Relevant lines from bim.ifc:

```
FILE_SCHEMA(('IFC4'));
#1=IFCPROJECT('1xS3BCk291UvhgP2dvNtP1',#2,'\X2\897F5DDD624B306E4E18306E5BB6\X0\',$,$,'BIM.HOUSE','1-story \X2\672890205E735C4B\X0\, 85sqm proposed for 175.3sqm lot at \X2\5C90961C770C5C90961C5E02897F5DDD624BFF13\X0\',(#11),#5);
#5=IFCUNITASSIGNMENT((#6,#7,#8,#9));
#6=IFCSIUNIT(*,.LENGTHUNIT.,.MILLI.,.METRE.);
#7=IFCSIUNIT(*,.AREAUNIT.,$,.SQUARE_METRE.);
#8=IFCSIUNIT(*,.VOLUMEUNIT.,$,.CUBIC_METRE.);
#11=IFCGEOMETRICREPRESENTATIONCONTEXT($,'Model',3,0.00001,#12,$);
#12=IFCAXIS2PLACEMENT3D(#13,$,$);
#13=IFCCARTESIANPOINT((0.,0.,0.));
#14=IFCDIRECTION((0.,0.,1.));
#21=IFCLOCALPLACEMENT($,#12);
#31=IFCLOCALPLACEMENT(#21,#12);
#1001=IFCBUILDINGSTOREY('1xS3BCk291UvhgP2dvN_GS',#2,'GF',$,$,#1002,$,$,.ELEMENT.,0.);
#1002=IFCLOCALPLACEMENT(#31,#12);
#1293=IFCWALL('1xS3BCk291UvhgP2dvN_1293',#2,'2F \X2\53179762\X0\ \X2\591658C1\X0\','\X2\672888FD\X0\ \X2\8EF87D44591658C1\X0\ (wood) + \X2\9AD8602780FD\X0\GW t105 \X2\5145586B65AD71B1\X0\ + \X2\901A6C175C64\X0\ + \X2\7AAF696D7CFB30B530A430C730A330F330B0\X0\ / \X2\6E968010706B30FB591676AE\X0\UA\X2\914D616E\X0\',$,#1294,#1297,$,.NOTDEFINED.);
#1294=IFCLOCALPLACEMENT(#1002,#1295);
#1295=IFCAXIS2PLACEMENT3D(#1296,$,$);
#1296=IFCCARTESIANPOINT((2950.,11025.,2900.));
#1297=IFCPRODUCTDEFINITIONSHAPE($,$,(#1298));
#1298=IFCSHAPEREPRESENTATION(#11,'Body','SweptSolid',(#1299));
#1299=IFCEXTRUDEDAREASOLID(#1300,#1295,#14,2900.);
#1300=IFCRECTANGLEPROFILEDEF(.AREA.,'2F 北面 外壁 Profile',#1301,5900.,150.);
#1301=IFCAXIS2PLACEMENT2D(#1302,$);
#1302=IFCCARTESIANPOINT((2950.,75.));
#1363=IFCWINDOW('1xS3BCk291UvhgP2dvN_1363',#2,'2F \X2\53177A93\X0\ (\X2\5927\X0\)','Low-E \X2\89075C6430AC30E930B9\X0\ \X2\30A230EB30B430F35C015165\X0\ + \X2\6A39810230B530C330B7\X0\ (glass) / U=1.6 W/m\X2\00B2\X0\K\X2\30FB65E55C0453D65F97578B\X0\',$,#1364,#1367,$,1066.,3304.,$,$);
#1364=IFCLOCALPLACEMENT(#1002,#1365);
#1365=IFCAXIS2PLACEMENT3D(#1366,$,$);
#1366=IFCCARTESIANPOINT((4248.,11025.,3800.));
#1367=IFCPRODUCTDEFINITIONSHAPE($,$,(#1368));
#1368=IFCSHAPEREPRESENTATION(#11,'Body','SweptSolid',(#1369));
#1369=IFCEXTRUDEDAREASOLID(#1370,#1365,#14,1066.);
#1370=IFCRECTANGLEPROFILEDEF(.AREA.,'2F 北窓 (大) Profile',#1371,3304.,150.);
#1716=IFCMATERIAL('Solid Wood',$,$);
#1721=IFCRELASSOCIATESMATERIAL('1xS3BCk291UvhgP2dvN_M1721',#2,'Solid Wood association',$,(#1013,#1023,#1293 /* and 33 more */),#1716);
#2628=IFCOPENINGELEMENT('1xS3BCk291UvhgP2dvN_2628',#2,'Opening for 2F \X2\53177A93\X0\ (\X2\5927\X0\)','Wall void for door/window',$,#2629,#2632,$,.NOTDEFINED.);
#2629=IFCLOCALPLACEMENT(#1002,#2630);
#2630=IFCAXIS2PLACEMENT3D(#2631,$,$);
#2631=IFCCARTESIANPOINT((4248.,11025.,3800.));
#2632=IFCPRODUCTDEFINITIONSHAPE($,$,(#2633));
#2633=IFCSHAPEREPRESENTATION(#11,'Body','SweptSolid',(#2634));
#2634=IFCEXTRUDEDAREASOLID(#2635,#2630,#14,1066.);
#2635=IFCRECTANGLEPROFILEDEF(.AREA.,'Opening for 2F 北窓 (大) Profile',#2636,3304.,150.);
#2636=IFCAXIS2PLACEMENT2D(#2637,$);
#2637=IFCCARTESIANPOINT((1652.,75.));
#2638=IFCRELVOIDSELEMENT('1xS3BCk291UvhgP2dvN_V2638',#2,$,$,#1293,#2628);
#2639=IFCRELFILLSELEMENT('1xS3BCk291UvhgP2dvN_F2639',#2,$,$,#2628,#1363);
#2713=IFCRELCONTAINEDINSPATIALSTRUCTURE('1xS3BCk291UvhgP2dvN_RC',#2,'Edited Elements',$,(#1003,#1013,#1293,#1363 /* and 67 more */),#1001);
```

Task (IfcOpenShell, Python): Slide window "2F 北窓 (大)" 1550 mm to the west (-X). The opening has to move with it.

```python
import ifcopenshell
import ifcopenshell.api.geometry
import ifcopenshell.util.placement
import ifcopenshell.util.unit

model = ifcopenshell.open("bim.ifc")
unit_scale = ifcopenshell.util.unit.calculate_unit_scale(model)

window = model.by_id(1363)
opening = window.FillsVoids[0].RelatingOpeningElement
wall = opening.VoidsElements[0].RelatingBuildingElement

wall_matrix = ifcopenshell.util.placement.get_local_placement(wall.ObjectPlacement)
shift = wall_matrix[:3, 0] * -1.55 / unit_scale
before = ifcopenshell.util.placement.get_local_placement(window.ObjectPlacement)[:3, 3].copy()

# The window is not placed relative to its opening, so move both.
for product in (opening, window):
    matrix = ifcopenshell.util.placement.get_local_placement(product.ObjectPlacement)
    matrix[:3, 3] += shift
    ifcopenshell.api.geometry.edit_object_placement(model, product=product, matrix=matrix, is_si=False)

after = ifcopenshell.util.placement.get_local_placement(window.ObjectPlacement)[:3, 3]
print("window moved by", (after - before).round(3) + 0.0)

model.write("bim-out.ifc")
```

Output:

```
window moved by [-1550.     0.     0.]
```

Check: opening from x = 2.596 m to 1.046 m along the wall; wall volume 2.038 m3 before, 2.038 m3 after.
